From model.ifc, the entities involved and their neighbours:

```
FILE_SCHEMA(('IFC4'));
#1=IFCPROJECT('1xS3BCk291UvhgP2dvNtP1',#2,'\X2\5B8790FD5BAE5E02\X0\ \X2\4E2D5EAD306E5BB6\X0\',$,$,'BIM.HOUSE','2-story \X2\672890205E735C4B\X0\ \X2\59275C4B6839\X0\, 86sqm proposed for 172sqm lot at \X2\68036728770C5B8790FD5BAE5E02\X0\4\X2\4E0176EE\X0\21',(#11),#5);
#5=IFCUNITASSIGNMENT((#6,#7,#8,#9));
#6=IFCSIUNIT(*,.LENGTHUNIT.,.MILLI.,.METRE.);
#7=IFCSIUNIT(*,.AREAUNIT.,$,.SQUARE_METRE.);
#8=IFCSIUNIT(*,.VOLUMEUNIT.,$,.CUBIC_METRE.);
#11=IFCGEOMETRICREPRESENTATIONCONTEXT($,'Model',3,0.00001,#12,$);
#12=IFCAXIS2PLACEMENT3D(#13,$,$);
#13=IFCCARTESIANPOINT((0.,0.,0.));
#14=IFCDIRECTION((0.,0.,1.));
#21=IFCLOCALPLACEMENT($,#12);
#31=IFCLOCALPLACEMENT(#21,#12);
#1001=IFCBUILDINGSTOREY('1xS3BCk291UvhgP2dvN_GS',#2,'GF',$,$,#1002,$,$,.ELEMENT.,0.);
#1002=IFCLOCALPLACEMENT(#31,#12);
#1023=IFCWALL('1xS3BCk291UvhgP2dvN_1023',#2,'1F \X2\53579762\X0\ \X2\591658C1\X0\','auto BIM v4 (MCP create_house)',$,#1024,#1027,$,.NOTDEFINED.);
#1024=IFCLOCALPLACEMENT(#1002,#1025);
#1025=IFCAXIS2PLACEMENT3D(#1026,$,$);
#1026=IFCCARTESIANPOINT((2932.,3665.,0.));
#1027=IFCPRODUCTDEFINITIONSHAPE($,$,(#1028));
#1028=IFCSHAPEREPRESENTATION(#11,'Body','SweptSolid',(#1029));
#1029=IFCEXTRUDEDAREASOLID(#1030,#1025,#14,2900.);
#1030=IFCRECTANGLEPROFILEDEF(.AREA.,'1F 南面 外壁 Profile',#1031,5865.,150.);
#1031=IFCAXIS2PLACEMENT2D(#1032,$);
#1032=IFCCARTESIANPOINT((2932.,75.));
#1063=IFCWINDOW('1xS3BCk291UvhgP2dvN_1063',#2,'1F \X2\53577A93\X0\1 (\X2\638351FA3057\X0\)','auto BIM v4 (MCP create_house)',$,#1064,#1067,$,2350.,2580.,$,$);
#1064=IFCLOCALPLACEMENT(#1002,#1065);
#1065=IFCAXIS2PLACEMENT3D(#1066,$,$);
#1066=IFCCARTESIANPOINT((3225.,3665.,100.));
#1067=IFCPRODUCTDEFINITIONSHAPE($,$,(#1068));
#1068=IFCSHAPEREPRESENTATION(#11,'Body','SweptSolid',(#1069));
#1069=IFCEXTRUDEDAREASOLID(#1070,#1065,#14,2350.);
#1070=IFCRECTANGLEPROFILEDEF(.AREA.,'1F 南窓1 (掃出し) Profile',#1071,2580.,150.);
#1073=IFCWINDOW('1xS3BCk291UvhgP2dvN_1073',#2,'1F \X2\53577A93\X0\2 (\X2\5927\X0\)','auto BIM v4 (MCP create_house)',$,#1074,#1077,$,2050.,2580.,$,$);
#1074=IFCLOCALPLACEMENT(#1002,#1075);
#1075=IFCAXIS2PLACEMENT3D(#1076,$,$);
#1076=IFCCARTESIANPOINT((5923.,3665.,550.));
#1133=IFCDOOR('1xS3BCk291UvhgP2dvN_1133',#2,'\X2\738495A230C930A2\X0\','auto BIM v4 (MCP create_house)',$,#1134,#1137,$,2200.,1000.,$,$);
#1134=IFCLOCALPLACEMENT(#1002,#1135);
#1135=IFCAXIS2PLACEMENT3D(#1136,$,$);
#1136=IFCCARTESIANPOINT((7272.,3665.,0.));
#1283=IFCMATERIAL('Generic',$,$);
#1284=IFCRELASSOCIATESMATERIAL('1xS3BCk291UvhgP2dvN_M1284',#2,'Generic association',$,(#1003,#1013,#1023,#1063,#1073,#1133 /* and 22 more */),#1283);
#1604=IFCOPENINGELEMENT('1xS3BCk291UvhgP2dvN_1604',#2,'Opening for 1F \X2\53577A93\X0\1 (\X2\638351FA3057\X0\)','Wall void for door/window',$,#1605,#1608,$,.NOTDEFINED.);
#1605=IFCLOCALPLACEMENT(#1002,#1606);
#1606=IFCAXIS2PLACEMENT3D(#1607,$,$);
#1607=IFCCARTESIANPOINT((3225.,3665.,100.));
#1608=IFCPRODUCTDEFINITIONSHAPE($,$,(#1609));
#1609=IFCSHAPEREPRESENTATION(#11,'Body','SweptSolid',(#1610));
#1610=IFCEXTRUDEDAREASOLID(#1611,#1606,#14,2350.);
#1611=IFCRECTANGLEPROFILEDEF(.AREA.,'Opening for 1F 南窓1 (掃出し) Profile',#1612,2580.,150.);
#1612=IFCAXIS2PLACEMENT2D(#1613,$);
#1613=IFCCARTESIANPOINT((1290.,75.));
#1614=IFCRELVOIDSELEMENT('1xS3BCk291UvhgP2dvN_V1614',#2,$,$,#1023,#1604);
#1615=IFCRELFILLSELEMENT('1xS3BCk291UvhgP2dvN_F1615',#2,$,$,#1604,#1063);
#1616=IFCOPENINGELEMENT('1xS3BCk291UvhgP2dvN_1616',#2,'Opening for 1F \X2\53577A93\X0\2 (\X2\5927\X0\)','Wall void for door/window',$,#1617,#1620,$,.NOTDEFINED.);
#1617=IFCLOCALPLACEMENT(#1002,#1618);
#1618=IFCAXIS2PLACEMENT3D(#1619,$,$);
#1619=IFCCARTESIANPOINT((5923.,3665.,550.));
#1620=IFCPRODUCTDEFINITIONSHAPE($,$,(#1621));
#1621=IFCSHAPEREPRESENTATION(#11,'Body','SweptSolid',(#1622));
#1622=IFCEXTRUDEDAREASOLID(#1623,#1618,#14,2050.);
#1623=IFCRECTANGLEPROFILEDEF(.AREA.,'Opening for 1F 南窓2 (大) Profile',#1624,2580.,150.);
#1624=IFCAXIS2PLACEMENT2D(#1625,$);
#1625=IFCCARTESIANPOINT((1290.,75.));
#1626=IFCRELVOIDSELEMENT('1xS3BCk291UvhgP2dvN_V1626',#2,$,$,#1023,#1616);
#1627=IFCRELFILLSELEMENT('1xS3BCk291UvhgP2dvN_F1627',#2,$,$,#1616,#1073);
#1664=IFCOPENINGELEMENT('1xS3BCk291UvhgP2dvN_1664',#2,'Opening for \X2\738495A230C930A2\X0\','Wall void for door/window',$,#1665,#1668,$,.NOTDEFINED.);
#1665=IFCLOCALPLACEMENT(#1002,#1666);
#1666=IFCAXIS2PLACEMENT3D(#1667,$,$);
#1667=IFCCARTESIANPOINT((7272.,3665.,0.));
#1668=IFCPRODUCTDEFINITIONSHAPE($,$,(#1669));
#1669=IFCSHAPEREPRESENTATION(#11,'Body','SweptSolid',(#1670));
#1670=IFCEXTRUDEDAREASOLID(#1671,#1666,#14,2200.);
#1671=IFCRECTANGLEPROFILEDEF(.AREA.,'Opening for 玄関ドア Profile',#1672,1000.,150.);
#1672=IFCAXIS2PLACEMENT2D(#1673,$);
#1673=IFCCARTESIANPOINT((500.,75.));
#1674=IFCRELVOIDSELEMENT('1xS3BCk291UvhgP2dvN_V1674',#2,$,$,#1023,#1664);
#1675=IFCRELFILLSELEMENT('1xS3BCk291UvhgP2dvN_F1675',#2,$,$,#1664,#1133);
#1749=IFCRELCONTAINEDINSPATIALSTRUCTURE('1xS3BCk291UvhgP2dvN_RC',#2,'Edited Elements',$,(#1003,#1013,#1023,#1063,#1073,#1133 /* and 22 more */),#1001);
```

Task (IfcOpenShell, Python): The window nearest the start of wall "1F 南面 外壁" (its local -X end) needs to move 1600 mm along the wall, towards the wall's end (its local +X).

```python
import ifcopenshell
import ifcopenshell.api.geometry
import ifcopenshell.util.placement

model = ifcopenshell.open("model.ifc")

window = model.by_id(1063)
opening = window.FillsVoids[0].RelatingOpeningElement
wall = opening.VoidsElements[0].RelatingBuildingElement

wall_matrix = ifcopenshell.util.placement.get_local_placement(wall.ObjectPlacement)
shift = wall_matrix[:3, 0] * 1600.0
before = ifcopenshell.util.placement.get_local_placement(window.ObjectPlacement)[:3, 3].copy()

# The window is not placed relative to its opening, so move both.
for product in (opening, window):
    matrix = ifcopenshell.util.placement.get_local_placement(product.ObjectPlacement)
    matrix[:3, 3] += shift
    ifcopenshell.api.geometry.edit_object_placement(model, product=product, matrix=matrix, is_si=False)

after = ifcopenshell.util.placement.get_local_placement(window.ObjectPlacement)[:3, 3]
print("window moved by", (after - before).round(3) + 0.0)

model.write("model_updated.ifc")
```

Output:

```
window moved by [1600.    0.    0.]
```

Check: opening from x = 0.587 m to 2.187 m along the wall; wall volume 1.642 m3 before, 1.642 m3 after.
